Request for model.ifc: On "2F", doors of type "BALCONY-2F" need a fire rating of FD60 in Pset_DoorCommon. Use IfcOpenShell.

First a look at what the model holds.

```python
import ifcopenshell
import ifcopenshell.util.element

model = ifcopenshell.open("model.ifc")
print(model.schema)
storey = next(s for s in model.by_type("IfcBuildingStorey") if s.Name == "2F")
doors = [e for e in ifcopenshell.util.element.get_decomposition(storey) if e.is_a("IfcDoor")]
seen = {}
for e in doors:
    element_type = ifcopenshell.util.element.get_type(e)
    key = (element_type.Name if element_type != e and element_type else None, ifcopenshell.util.element.get_pset(e, "Pset_DoorCommon", "FireRating"))
    seen[key] = seen.get(key, 0) + 1
for (name, value), count in sorted(seen.items(), key=str):
    print(count, "x", name, "|", value)
```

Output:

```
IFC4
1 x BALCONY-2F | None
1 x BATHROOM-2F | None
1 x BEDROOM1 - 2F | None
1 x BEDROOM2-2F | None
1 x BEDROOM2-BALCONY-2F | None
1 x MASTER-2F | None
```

```python
import ifcopenshell
import ifcopenshell.api.pset
import ifcopenshell.util.element

model = ifcopenshell.open("model.ifc")

storey = next(s for s in model.by_type("IfcBuildingStorey") if s.Name == "2F")
doors = [e for e in ifcopenshell.util.element.get_decomposition(storey) if e.is_a("IfcDoor")]

count = 0
for e in doors:
    element_type = ifcopenshell.util.element.get_type(e)
    if element_type in (None, e) or element_type.Name != "BALCONY-2F":
        continue
    # add_pset returns the element's existing set when there is one.
    pset = ifcopenshell.api.pset.add_pset(model, product=e, name="Pset_DoorCommon")
    ifcopenshell.api.pset.edit_pset(model, pset=pset, properties={"FireRating": "FD60"})
    count += 1

print(count, "doors updated")

model.write("model-out.ifc")
```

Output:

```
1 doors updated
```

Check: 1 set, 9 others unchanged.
